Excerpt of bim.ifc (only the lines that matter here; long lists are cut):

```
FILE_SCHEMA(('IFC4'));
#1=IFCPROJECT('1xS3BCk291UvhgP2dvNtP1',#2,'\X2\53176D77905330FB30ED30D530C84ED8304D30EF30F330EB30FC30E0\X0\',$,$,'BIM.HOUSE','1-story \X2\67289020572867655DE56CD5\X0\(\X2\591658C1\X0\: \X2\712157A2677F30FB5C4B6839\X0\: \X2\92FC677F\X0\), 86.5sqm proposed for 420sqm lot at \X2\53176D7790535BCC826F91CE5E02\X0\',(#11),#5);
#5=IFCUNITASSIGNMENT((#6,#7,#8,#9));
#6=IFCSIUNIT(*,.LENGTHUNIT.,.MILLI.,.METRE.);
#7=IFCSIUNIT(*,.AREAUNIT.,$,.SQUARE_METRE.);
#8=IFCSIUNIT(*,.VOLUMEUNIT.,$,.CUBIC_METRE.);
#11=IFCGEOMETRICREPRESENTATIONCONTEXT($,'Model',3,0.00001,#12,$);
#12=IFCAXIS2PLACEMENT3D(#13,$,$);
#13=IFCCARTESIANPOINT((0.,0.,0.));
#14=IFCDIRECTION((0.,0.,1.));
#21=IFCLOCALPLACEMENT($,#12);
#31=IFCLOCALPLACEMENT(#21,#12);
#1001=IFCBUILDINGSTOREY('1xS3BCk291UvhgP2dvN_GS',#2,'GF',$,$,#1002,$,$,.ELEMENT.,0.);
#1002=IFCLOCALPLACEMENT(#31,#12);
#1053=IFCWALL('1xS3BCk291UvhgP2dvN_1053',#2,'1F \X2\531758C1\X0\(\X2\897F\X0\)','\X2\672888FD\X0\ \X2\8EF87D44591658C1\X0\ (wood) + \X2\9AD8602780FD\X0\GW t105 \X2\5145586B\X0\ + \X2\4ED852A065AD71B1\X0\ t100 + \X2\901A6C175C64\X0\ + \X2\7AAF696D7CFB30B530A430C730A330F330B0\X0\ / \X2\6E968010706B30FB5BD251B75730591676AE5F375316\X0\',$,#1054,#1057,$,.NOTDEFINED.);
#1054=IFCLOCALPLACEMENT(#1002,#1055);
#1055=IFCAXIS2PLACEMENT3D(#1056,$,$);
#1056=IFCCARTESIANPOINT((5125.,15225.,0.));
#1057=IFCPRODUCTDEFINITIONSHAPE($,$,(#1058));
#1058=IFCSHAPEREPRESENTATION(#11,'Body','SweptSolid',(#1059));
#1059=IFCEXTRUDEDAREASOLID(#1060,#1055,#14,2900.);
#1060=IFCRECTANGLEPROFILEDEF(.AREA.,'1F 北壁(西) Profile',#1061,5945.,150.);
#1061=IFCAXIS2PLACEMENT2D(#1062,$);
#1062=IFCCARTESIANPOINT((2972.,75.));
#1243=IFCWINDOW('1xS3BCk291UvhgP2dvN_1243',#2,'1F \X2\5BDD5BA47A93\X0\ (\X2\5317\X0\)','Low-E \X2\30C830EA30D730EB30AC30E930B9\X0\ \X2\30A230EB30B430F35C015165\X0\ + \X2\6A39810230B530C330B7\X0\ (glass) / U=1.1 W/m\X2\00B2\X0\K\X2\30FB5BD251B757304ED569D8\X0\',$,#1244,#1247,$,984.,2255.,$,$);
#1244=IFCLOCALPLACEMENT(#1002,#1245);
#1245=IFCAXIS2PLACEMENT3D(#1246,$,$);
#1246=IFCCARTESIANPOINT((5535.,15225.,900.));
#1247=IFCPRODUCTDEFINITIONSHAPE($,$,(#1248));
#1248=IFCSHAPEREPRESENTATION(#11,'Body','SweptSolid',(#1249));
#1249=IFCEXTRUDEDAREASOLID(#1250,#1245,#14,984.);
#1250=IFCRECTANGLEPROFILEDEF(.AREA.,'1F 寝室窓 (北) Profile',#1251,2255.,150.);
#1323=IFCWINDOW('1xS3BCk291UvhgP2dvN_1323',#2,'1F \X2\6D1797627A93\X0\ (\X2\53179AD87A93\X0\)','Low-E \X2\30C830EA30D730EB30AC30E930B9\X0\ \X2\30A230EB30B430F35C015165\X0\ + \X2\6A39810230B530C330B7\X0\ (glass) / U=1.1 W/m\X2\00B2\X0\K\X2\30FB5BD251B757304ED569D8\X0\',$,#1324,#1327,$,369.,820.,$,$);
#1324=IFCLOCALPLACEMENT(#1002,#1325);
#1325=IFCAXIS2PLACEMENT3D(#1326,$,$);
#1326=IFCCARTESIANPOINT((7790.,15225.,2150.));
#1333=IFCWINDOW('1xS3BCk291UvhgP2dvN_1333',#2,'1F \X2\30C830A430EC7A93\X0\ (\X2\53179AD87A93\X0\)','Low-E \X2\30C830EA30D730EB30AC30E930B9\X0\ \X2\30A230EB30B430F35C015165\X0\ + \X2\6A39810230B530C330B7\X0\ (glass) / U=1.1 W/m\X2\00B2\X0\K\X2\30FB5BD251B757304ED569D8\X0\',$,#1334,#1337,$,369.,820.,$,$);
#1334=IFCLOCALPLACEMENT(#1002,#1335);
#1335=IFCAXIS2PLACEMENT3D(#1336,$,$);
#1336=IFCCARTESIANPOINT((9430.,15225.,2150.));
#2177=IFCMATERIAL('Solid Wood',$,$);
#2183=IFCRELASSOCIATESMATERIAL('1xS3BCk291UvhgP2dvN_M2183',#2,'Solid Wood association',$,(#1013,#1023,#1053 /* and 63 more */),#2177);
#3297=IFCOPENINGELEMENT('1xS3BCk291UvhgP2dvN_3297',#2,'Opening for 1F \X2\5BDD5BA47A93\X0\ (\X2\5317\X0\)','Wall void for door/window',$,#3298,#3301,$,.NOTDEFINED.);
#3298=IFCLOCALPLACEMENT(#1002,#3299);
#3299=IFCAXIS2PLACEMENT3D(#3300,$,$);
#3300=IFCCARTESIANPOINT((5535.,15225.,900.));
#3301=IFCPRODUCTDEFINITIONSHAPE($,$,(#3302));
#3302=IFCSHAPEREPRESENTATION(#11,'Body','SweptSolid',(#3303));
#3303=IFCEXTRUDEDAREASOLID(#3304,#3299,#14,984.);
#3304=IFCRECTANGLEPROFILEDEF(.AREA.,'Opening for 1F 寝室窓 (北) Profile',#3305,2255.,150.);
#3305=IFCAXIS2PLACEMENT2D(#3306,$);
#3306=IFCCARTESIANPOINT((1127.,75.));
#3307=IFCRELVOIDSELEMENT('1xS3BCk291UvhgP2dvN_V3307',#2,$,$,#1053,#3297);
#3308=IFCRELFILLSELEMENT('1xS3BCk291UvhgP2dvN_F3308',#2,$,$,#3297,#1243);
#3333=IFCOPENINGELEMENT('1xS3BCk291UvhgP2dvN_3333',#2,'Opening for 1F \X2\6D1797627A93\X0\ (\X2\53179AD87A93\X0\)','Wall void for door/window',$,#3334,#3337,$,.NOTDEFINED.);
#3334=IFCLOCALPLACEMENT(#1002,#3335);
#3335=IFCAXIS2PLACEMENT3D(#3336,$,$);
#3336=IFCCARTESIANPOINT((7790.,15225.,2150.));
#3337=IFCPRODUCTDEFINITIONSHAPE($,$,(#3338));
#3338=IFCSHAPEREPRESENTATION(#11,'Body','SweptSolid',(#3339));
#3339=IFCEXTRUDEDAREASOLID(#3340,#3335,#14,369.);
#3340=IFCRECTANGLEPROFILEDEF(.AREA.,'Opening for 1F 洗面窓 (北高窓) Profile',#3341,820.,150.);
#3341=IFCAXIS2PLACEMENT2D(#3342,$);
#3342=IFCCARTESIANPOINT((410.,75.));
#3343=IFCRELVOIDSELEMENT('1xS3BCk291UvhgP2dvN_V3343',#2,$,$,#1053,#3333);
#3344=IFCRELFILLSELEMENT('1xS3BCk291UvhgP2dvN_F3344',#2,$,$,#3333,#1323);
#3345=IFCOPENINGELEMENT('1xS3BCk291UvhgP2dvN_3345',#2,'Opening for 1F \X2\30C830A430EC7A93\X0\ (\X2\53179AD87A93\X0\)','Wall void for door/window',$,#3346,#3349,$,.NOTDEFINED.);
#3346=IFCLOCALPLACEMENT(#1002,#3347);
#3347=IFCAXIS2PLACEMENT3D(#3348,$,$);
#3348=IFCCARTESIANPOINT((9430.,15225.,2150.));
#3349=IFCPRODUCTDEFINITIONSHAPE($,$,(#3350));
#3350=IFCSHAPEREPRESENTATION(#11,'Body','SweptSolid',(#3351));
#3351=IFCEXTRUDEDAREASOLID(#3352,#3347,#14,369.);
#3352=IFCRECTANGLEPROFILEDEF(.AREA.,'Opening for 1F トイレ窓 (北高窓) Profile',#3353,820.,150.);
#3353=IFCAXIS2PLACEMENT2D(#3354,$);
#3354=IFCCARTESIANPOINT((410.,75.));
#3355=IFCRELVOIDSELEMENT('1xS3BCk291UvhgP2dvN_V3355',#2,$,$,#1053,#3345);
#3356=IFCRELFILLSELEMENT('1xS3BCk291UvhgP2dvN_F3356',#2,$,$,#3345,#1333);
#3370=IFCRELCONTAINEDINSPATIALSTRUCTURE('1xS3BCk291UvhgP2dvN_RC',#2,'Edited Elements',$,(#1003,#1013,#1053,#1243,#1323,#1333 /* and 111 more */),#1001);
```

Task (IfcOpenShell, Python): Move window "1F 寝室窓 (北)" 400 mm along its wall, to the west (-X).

```python
import ifcopenshell
import ifcopenshell.api.geometry
import ifcopenshell.util.placement
import ifcopenshell.util.unit

model = ifcopenshell.open("bim.ifc")
unit_scale = ifcopenshell.util.unit.calculate_unit_scale(model)

window = model.by_guid("1xS3BCk291UvhgP2dvN_1243")
opening = window.FillsVoids[0].RelatingOpeningElement
wall = opening.VoidsElements[0].RelatingBuildingElement

wall_matrix = ifcopenshell.util.placement.get_local_placement(wall.ObjectPlacement)
shift = wall_matrix[:3, 0] * -0.4 / unit_scale
before = ifcopenshell.util.placement.get_local_placement(window.ObjectPlacement)[:3, 3].copy()

# The window is not placed relative to its opening, so move both.
for product in (opening, window):
    matrix = ifcopenshell.util.placement.get_local_placement(product.ObjectPlacement)
    matrix[:3, 3] += shift
    ifcopenshell.api.geometry.edit_object_placement(model, product=product, matrix=matrix, is_si=False)

after = ifcopenshell.util.placement.get_local_placement(window.ObjectPlacement)[:3, 3]
print("window moved by", (after - before).round(3) + 0.0)

model.write("bim_v2.ifc")
```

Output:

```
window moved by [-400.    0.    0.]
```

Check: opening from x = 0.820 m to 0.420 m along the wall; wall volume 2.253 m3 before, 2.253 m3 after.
